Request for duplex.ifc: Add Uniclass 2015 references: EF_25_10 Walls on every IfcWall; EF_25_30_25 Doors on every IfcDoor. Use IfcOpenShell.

First a look at what the model holds.

```python
import ifcopenshell

model = ifcopenshell.open("duplex.ifc")
print(model.schema)
print("classifications:", [c.Name for c in model.by_type("IfcClassification")])
for ifc_class in ("IfcDoor", "IfcRoof", "IfcStair", "IfcWall", "IfcWindow"):
    print(ifc_class, len(model.by_type(ifc_class)))
```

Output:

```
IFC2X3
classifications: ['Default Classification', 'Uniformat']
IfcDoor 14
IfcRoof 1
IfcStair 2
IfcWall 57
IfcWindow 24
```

```python
import ifcopenshell
import ifcopenshell.api.classification

model = ifcopenshell.open("duplex.ifc")

# IFC2X3 requires Source and Edition and has no link from the project to the system.
system = model.create_entity("IfcClassification", Source="NBS", Edition="2015", Name="Uniclass 2015")

codes = {
    "IfcWall": ("EF_25_10", "Walls"),
    "IfcDoor": ("EF_25_30_25", "Doors"),
}
for ifc_class, (code, name) in codes.items():
    products = model.by_type(ifc_class)
    ifcopenshell.api.classification.add_reference(
        model, products=products, classification=system, identification=code, name=name
    )
    print(code, len(products))

model.write("duplex_v2.ifc")
```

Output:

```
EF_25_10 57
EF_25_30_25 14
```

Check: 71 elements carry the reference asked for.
